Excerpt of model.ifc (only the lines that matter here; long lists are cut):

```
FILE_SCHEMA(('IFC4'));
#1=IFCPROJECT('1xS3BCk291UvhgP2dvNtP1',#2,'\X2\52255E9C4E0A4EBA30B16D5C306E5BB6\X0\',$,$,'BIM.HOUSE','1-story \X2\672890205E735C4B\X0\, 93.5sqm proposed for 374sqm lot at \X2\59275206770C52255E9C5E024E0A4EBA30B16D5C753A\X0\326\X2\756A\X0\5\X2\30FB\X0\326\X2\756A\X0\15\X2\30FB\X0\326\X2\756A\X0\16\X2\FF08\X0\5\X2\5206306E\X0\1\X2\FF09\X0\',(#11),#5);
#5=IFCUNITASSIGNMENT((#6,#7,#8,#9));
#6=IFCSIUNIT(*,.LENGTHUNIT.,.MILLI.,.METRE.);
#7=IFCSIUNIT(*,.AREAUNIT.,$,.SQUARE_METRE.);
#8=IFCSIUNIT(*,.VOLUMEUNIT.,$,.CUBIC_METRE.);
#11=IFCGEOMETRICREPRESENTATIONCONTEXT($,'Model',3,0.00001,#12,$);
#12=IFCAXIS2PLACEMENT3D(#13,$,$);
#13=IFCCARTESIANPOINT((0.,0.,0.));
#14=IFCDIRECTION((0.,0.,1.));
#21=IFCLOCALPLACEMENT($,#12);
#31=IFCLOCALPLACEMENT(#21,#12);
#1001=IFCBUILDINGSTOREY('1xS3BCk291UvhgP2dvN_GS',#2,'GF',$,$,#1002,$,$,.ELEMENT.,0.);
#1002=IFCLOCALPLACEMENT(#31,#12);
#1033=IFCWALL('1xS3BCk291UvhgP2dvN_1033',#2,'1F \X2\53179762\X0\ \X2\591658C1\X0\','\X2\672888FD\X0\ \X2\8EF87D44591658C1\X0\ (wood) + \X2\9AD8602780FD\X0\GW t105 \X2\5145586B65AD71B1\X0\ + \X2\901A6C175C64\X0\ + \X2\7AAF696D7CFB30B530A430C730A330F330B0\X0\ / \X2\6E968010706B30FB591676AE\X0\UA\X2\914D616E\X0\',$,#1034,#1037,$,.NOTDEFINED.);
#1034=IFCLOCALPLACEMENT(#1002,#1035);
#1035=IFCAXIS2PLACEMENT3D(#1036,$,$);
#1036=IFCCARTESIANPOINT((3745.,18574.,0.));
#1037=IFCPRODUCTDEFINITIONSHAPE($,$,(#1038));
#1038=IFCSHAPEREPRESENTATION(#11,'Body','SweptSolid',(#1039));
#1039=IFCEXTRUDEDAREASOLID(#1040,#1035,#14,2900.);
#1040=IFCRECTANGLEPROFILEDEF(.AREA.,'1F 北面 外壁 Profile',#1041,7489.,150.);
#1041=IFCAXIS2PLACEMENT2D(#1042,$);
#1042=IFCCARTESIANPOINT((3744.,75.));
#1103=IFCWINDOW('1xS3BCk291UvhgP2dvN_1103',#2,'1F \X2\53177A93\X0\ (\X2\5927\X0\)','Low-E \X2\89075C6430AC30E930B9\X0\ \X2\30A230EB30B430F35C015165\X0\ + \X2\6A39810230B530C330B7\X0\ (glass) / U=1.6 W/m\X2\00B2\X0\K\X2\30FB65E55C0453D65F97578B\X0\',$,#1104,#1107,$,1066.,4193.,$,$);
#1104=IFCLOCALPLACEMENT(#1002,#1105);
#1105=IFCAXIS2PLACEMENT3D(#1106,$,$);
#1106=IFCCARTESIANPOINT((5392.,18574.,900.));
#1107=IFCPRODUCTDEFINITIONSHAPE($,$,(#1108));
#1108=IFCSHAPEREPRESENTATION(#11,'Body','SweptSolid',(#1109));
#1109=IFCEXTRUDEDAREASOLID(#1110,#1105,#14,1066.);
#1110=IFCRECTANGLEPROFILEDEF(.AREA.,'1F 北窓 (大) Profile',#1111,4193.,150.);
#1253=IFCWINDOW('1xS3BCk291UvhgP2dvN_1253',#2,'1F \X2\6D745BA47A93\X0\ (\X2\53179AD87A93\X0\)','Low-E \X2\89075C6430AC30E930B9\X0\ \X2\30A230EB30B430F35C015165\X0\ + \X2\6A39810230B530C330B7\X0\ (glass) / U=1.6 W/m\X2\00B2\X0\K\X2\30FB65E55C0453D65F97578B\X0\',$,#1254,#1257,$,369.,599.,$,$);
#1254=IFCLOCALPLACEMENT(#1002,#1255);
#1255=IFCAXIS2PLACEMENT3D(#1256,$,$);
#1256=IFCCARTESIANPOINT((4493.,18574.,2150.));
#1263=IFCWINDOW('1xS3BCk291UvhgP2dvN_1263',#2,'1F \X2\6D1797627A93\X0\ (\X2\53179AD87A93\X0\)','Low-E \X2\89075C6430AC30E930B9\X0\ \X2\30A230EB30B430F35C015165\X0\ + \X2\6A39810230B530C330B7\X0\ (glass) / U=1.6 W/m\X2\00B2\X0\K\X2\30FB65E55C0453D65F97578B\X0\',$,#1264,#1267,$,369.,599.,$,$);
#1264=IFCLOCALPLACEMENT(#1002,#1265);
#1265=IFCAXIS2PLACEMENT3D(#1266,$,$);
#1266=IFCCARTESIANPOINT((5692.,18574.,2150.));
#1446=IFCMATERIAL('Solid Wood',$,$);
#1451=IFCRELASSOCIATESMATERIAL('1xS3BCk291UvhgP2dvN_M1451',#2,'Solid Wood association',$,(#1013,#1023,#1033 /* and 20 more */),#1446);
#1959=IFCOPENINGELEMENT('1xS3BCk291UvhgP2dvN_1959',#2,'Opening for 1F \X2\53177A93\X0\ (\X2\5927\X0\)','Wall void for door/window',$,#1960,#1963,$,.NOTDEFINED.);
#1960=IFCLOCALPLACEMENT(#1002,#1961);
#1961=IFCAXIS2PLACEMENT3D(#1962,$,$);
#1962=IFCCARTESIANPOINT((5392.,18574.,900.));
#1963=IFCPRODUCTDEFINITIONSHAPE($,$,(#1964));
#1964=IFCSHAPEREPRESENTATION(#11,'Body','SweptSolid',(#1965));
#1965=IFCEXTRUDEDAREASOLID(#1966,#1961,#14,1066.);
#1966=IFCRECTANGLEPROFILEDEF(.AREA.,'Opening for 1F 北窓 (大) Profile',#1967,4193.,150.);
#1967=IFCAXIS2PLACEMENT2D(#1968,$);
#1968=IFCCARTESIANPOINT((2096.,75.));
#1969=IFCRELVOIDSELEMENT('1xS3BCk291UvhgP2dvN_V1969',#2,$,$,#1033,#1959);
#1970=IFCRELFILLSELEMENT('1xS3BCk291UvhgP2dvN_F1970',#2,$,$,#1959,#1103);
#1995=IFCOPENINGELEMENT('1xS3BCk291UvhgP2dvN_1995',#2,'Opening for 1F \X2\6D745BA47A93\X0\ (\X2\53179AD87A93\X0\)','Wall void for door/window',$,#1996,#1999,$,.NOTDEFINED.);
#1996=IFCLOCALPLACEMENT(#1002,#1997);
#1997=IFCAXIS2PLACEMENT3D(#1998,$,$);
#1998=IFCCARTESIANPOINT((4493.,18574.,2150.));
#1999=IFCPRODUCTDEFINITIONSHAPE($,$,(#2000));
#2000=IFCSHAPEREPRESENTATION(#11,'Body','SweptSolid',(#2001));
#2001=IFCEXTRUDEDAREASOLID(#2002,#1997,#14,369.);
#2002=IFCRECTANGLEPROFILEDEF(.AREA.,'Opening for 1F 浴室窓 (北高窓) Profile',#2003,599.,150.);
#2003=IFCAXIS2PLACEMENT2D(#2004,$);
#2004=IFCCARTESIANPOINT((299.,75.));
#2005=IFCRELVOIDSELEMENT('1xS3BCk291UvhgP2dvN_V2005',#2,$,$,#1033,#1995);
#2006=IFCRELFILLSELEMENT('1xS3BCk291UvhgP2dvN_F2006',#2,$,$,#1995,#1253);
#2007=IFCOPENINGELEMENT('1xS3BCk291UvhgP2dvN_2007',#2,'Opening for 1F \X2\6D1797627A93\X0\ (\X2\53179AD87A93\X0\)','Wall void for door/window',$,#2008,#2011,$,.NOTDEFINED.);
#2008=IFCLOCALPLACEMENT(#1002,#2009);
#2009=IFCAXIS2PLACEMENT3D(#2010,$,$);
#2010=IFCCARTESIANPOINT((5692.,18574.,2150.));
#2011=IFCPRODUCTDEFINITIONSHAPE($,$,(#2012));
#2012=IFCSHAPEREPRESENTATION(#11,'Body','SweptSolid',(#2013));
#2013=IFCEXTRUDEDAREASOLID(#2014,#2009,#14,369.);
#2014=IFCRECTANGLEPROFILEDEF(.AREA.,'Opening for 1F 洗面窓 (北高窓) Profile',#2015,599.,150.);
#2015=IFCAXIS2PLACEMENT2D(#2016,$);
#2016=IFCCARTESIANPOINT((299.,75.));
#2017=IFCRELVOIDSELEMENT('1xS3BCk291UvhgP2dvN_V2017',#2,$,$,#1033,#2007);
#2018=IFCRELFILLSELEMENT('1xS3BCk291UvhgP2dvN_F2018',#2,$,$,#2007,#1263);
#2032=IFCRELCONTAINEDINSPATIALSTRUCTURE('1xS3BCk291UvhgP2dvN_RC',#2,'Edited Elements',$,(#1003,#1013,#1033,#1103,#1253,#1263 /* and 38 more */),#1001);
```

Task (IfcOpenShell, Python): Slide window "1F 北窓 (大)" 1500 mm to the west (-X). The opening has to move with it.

```python
import ifcopenshell
import ifcopenshell.api.geometry
import ifcopenshell.util.placement
import ifcopenshell.util.unit

model = ifcopenshell.open("model.ifc")
unit_scale = ifcopenshell.util.unit.calculate_unit_scale(model)

window = model.by_id(1103)
opening = window.FillsVoids[0].RelatingOpeningElement
wall = opening.VoidsElements[0].RelatingBuildingElement

wall_matrix = ifcopenshell.util.placement.get_local_placement(wall.ObjectPlacement)
shift = wall_matrix[:3, 0] * -1.5 / unit_scale
before = ifcopenshell.util.placement.get_local_placement(window.ObjectPlacement)[:3, 3].copy()

# The window is not placed relative to its opening, so move both.
for product in (opening, window):
    matrix = ifcopenshell.util.placement.get_local_placement(product.ObjectPlacement)
    matrix[:3, 3] += shift
    ifcopenshell.api.geometry.edit_object_placement(model, product=product, matrix=matrix, is_si=False)

after = ifcopenshell.util.placement.get_local_placement(window.ObjectPlacement)[:3, 3]
print("window moved by", (after - before).round(3) + 0.0)

model.write("model_edited.ifc")
```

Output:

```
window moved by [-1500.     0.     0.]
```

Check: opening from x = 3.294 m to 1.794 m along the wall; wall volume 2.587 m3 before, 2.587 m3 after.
